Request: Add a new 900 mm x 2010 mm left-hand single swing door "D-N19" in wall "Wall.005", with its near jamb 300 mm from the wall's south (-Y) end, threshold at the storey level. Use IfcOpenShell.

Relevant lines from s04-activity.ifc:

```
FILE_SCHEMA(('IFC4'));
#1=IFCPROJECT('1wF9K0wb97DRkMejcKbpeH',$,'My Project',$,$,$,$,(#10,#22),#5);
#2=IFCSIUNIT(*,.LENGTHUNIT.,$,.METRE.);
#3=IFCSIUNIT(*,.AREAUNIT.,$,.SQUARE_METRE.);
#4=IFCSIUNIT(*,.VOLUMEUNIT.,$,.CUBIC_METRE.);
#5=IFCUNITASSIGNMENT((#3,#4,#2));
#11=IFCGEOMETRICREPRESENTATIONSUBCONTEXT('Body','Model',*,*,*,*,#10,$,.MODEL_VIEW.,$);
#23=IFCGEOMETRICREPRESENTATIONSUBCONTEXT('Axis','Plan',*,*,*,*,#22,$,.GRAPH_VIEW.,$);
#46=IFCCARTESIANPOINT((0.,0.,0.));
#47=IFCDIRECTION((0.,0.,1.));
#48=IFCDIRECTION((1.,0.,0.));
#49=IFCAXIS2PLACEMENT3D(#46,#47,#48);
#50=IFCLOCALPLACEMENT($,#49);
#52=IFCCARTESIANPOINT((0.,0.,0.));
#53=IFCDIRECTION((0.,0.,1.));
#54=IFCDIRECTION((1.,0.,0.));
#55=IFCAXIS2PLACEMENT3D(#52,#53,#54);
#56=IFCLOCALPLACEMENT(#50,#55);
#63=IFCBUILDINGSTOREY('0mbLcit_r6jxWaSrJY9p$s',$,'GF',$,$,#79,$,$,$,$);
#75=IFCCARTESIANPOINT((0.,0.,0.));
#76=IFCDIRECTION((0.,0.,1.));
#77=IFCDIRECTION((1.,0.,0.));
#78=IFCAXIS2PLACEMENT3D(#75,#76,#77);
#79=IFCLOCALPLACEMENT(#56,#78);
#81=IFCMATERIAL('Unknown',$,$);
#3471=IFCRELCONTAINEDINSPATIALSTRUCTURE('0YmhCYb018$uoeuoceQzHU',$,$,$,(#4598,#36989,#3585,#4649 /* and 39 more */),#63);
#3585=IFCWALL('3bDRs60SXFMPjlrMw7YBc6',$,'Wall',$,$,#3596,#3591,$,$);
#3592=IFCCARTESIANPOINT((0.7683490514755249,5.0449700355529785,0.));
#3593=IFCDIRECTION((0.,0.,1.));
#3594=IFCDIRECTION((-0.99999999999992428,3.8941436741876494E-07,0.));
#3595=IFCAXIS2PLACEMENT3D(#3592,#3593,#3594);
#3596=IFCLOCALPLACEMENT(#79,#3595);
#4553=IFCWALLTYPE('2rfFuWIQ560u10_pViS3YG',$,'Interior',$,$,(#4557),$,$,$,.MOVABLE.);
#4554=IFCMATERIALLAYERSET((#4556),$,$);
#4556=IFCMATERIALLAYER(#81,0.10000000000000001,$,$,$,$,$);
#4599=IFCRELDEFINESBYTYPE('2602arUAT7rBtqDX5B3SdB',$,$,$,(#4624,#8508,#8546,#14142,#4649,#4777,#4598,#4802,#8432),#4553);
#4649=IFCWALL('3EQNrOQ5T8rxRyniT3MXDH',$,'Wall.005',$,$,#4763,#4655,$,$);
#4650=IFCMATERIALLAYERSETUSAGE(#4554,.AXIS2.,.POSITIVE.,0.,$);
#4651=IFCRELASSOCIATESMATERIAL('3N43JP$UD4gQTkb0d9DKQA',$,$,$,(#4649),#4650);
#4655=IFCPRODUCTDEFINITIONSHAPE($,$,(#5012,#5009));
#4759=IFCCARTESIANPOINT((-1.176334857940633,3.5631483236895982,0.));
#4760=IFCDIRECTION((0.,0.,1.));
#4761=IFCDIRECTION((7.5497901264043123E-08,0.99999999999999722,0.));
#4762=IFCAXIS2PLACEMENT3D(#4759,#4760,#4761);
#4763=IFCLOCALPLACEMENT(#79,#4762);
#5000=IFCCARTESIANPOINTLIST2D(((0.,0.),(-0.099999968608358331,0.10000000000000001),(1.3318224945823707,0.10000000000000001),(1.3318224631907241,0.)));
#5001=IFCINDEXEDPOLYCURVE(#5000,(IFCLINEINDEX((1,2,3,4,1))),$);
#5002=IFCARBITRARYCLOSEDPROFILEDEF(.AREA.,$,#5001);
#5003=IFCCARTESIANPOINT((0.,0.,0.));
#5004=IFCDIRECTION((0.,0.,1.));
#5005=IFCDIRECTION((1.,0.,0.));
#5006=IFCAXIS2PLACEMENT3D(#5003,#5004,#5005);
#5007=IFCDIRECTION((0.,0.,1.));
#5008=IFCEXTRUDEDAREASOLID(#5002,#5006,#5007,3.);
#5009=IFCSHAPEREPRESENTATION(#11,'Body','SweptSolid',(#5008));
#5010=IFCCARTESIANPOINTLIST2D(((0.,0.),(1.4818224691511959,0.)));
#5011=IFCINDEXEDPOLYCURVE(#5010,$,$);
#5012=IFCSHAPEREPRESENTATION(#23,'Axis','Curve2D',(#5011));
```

```python
import numpy as np
import ifcopenshell
import ifcopenshell.api.feature
import ifcopenshell.api.geometry
import ifcopenshell.api.root
import ifcopenshell.api.spatial
import ifcopenshell.geom
import ifcopenshell.util.element
import ifcopenshell.util.placement
import ifcopenshell.util.representation
import ifcopenshell.util.shape
import ifcopenshell.util.unit

model = ifcopenshell.open("s04-activity.ifc")
unit_scale = ifcopenshell.util.unit.calculate_unit_scale(model)
settings = ifcopenshell.geom.settings()


def volume(element):
    """Net volume in cubic metres, openings subtracted."""
    shape = ifcopenshell.geom.create_shape(settings, element)
    return ifcopenshell.util.shape.get_volume(shape.geometry)


wall = model.by_guid("3EQNrOQ5T8rxRyniT3MXDH")
storey = ifcopenshell.util.element.get_container(wall, ifc_class="IfcBuildingStorey")
context = ifcopenshell.util.representation.get_context(model, "Model", "Body", "MODEL_VIEW")
before = volume(wall)

width, height, from_end, sill = 0.9, 2.01, 0.3, 0.0  # metres

# The wall runs along its own X axis, and the end named is its -X end.
wall_shape = ifcopenshell.geom.create_shape(settings, wall)
x, y, z = ifcopenshell.util.shape.get_vertices(wall_shape.geometry).T
start = x.min() + from_end
face, thickness = float(y.min()), float(y.max() - y.min())
wall_matrix = ifcopenshell.util.placement.get_local_placement(wall.ObjectPlacement)
level = ifcopenshell.util.placement.get_local_placement(storey.ObjectPlacement)[2, 3]


def in_wall(x, y):
    """Placement at x, y metres in the wall's axes, at sill height."""
    matrix = wall_matrix.copy()
    matrix[:, 3] = wall_matrix @ np.array([x / unit_scale, y / unit_scale, 0.0, 1.0])
    matrix[2, 3] = level + sill / unit_scale
    return matrix


# Opening: a box that overshoots both wall faces by 50 mm.
opening = ifcopenshell.api.root.create_entity(model, ifc_class="IfcOpeningElement", predefined_type="OPENING")
box = ifcopenshell.api.geometry.add_wall_representation(
    model, context=context, length=width, height=height, thickness=thickness + 0.1
)
ifcopenshell.api.geometry.assign_representation(model, product=opening, representation=box)
ifcopenshell.api.geometry.edit_object_placement(model, product=opening, matrix=in_wall(start, face - 0.05), is_si=False)
ifcopenshell.api.feature.add_feature(model, feature=opening, element=wall)

door = ifcopenshell.api.root.create_entity(model, ifc_class="IfcDoor", name="D-N19", predefined_type="DOOR")
door.OverallWidth, door.OverallHeight = width / unit_scale, height / unit_scale
door.OperationType = "SINGLE_SWING_LEFT"
body = ifcopenshell.api.geometry.add_door_representation(
    model,
    context=context,
    overall_width=door.OverallWidth,
    overall_height=door.OverallHeight,
    operation_type="SINGLE_SWING_LEFT",
    lining_properties={"LiningDepth": thickness / unit_scale, "ThresholdDepth": thickness / unit_scale},
)
ifcopenshell.api.geometry.assign_representation(model, product=door, representation=body)
ifcopenshell.api.spatial.assign_container(model, products=[door], relating_structure=storey)
ifcopenshell.api.feature.add_filling(model, opening=opening, element=door)

# The lining spans the wall, so the door starts at the wall face.
ifcopenshell.api.geometry.edit_object_placement(model, product=door, matrix=in_wall(start, face), is_si=False)

after = volume(wall)

print(f"wall volume {before:.3f} -> {after:.3f} m3")

model.write("s04-activity-out.ifc")
```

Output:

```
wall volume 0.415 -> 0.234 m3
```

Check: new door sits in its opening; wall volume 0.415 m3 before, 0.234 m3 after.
